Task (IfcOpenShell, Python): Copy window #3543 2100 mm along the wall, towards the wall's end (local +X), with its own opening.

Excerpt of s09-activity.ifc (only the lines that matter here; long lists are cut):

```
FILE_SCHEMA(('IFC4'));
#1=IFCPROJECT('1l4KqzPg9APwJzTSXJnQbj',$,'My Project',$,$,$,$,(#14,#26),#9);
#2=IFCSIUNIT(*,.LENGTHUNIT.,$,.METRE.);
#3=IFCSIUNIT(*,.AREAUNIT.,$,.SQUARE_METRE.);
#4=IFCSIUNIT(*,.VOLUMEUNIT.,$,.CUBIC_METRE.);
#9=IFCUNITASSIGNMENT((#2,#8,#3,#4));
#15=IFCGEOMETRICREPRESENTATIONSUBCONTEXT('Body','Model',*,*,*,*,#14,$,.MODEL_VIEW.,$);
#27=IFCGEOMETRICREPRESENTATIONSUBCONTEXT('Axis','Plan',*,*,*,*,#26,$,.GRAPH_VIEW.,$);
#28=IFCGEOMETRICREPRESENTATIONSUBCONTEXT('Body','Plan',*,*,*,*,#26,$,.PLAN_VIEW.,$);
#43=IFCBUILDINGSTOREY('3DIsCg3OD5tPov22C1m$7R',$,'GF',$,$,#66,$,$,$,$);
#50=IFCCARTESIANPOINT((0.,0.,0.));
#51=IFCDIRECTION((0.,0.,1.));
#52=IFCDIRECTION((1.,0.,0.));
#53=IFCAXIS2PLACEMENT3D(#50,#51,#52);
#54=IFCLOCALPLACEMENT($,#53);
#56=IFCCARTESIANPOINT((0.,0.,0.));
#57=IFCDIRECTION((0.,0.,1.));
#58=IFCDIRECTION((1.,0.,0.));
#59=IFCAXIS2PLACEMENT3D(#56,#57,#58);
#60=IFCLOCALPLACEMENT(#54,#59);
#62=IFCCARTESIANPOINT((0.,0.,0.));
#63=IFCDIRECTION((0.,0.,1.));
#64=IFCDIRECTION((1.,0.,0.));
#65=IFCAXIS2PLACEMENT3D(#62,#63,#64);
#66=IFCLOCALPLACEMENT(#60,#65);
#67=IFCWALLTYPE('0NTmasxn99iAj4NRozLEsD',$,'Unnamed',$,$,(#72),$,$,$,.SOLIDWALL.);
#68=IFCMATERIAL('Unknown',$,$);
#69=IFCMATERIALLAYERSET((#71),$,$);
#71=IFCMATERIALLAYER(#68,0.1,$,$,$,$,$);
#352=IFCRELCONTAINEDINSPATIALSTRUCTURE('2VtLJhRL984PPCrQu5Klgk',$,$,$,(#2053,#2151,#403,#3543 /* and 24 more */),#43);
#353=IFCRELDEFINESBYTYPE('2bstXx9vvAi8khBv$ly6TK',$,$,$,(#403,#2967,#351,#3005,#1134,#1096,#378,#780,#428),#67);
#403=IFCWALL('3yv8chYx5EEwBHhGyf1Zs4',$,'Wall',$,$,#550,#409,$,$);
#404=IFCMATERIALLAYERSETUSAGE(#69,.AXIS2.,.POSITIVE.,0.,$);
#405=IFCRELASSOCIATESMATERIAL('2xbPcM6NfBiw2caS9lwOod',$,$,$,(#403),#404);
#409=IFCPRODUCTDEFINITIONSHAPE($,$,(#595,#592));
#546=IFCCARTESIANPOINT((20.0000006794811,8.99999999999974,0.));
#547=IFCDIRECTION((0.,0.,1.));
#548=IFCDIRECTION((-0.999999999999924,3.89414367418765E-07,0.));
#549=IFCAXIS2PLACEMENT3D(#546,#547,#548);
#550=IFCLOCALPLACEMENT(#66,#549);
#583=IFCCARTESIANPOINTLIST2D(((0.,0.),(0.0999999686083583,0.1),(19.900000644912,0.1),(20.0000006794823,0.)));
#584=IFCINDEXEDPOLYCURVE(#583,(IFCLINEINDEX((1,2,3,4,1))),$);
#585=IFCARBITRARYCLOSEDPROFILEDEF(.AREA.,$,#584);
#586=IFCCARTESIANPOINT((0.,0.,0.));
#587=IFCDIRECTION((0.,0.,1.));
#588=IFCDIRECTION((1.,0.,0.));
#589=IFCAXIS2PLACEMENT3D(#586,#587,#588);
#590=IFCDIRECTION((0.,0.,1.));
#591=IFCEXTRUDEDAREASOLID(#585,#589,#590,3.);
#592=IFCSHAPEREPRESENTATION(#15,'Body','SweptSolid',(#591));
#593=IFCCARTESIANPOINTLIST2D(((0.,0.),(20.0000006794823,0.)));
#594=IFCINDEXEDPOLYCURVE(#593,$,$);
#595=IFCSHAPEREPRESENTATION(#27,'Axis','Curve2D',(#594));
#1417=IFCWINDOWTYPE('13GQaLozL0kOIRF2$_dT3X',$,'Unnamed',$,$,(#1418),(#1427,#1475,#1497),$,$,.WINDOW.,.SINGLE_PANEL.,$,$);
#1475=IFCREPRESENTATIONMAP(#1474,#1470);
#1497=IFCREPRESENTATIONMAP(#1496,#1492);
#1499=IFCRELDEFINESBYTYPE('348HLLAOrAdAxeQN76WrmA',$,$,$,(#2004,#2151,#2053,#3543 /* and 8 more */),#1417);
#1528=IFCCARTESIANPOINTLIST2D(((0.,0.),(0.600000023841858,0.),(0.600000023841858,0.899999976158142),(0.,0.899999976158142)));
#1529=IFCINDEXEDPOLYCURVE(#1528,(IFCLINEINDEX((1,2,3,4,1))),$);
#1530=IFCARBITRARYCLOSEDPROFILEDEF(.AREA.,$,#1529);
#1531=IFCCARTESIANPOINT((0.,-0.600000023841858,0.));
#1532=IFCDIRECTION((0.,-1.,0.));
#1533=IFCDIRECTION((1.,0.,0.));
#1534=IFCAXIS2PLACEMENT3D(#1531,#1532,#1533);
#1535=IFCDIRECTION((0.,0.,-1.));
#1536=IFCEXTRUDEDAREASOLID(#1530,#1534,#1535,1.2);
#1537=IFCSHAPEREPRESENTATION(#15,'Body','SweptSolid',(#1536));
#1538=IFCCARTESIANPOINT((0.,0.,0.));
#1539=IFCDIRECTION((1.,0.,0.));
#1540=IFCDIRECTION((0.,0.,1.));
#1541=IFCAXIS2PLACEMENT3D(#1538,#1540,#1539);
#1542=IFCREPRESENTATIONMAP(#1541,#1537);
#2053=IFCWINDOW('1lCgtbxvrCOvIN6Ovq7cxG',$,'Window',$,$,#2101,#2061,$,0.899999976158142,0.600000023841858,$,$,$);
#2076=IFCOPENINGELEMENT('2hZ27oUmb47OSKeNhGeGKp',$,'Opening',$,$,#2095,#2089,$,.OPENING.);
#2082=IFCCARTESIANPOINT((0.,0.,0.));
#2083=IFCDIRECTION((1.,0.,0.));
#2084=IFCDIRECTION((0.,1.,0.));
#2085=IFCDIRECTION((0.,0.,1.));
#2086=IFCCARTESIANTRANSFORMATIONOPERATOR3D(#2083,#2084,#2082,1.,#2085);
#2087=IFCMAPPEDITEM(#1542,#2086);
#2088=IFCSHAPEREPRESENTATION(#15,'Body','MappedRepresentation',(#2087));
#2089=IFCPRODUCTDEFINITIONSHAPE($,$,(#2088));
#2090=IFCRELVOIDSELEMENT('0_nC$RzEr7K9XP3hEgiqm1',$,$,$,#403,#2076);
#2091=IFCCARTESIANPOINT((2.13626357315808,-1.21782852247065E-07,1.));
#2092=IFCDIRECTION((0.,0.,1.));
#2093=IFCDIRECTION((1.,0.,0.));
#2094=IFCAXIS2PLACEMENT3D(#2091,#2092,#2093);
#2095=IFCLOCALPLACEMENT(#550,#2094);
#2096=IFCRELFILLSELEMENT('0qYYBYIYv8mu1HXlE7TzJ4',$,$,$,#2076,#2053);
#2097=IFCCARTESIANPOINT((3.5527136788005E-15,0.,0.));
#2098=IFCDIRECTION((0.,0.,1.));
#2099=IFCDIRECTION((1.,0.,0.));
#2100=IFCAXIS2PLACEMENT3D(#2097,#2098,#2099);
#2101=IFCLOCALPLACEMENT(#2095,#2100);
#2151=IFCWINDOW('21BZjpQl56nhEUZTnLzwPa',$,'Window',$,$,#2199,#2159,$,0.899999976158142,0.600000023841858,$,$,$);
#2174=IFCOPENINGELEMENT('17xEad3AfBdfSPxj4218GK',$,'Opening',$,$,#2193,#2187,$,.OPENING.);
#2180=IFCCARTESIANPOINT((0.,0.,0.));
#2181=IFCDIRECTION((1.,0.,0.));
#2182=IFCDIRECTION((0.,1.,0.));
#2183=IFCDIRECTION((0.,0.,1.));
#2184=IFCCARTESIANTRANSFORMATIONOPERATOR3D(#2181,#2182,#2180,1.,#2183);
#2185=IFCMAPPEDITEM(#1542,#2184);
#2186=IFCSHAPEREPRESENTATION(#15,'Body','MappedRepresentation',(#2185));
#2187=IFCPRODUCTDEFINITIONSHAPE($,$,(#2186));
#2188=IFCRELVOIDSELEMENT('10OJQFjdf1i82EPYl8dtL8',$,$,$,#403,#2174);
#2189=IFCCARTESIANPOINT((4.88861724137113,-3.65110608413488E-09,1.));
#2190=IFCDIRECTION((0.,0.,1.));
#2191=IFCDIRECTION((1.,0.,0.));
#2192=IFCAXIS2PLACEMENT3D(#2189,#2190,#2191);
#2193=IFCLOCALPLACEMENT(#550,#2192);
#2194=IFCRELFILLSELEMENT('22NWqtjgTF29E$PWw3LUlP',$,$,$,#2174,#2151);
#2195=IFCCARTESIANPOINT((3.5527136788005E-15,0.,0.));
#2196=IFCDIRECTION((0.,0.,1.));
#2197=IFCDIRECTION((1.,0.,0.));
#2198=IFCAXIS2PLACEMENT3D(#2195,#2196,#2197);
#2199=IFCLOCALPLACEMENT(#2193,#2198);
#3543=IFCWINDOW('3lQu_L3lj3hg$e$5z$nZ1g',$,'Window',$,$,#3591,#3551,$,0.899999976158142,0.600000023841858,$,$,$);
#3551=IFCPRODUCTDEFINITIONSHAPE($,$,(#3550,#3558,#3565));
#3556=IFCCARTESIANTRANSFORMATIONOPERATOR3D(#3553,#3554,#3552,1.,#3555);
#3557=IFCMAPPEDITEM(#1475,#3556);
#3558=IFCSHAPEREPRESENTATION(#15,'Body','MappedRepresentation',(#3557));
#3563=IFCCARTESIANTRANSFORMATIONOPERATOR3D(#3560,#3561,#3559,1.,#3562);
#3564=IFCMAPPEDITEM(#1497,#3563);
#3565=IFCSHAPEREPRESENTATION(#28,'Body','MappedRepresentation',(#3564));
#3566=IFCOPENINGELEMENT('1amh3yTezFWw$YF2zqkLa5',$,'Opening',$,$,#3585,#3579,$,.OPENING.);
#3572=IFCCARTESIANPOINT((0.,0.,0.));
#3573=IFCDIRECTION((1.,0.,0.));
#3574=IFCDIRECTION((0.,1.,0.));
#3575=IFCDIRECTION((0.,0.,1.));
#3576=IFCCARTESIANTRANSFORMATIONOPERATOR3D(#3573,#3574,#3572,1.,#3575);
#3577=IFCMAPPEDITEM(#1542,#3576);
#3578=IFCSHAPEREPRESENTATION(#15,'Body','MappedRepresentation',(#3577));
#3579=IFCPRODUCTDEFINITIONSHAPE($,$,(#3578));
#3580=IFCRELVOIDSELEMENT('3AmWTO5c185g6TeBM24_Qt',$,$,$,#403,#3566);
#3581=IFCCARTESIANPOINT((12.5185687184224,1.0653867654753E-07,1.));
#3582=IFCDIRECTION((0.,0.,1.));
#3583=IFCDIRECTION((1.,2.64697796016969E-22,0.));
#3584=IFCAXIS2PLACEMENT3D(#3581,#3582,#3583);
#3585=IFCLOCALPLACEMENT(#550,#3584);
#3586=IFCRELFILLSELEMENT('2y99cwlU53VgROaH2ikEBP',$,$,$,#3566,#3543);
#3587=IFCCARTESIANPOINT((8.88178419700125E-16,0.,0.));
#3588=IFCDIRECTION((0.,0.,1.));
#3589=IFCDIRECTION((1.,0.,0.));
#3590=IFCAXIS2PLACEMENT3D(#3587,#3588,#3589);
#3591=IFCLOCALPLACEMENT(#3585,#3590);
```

```python
import ifcopenshell
import ifcopenshell.api.feature
import ifcopenshell.api.geometry
import ifcopenshell.api.root
import ifcopenshell.geom
import ifcopenshell.util.element
import ifcopenshell.util.placement
import ifcopenshell.util.shape
import ifcopenshell.util.unit

model = ifcopenshell.open("s09-activity.ifc")
unit_scale = ifcopenshell.util.unit.calculate_unit_scale(model)
settings = ifcopenshell.geom.settings()


def volume(element):
    """Net volume in cubic metres, openings subtracted."""
    shape = ifcopenshell.geom.create_shape(settings, element)
    return ifcopenshell.util.shape.get_volume(shape.geometry)


window = model.by_id(3543)
opening = window.FillsVoids[0].RelatingOpeningElement
wall = opening.VoidsElements[0].RelatingBuildingElement
before = volume(wall)
shift = ifcopenshell.util.placement.get_local_placement(wall.ObjectPlacement)[:3, 0] * 2.1 / unit_scale

# copy_class copies the void relationship, type, container and properties, but no geometry.
new_opening = ifcopenshell.api.root.copy_class(model, product=opening)
new_opening.Representation = ifcopenshell.util.element.copy_deep(
    model, opening.Representation, exclude=["IfcGeometricRepresentationContext", "IfcRepresentationMap"]
)
new_window = ifcopenshell.api.root.copy_class(model, product=window)
new_window.Representation = ifcopenshell.util.element.copy_deep(
    model, window.Representation, exclude=["IfcGeometricRepresentationContext", "IfcRepresentationMap"]
)
ifcopenshell.api.feature.add_filling(model, opening=new_opening, element=new_window)

for old, new in ((opening, new_opening), (window, new_window)):
    matrix = ifcopenshell.util.placement.get_local_placement(old.ObjectPlacement)
    matrix[:3, 3] += shift
    ifcopenshell.api.geometry.edit_object_placement(model, product=new, matrix=matrix, is_si=False)

after = volume(wall)

print(f"wall volume {before:.3f} -> {after:.3f} m3")

model.write("s09-activity-out.ifc")
```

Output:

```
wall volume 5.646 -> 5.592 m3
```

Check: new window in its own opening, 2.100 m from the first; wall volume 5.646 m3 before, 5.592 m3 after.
